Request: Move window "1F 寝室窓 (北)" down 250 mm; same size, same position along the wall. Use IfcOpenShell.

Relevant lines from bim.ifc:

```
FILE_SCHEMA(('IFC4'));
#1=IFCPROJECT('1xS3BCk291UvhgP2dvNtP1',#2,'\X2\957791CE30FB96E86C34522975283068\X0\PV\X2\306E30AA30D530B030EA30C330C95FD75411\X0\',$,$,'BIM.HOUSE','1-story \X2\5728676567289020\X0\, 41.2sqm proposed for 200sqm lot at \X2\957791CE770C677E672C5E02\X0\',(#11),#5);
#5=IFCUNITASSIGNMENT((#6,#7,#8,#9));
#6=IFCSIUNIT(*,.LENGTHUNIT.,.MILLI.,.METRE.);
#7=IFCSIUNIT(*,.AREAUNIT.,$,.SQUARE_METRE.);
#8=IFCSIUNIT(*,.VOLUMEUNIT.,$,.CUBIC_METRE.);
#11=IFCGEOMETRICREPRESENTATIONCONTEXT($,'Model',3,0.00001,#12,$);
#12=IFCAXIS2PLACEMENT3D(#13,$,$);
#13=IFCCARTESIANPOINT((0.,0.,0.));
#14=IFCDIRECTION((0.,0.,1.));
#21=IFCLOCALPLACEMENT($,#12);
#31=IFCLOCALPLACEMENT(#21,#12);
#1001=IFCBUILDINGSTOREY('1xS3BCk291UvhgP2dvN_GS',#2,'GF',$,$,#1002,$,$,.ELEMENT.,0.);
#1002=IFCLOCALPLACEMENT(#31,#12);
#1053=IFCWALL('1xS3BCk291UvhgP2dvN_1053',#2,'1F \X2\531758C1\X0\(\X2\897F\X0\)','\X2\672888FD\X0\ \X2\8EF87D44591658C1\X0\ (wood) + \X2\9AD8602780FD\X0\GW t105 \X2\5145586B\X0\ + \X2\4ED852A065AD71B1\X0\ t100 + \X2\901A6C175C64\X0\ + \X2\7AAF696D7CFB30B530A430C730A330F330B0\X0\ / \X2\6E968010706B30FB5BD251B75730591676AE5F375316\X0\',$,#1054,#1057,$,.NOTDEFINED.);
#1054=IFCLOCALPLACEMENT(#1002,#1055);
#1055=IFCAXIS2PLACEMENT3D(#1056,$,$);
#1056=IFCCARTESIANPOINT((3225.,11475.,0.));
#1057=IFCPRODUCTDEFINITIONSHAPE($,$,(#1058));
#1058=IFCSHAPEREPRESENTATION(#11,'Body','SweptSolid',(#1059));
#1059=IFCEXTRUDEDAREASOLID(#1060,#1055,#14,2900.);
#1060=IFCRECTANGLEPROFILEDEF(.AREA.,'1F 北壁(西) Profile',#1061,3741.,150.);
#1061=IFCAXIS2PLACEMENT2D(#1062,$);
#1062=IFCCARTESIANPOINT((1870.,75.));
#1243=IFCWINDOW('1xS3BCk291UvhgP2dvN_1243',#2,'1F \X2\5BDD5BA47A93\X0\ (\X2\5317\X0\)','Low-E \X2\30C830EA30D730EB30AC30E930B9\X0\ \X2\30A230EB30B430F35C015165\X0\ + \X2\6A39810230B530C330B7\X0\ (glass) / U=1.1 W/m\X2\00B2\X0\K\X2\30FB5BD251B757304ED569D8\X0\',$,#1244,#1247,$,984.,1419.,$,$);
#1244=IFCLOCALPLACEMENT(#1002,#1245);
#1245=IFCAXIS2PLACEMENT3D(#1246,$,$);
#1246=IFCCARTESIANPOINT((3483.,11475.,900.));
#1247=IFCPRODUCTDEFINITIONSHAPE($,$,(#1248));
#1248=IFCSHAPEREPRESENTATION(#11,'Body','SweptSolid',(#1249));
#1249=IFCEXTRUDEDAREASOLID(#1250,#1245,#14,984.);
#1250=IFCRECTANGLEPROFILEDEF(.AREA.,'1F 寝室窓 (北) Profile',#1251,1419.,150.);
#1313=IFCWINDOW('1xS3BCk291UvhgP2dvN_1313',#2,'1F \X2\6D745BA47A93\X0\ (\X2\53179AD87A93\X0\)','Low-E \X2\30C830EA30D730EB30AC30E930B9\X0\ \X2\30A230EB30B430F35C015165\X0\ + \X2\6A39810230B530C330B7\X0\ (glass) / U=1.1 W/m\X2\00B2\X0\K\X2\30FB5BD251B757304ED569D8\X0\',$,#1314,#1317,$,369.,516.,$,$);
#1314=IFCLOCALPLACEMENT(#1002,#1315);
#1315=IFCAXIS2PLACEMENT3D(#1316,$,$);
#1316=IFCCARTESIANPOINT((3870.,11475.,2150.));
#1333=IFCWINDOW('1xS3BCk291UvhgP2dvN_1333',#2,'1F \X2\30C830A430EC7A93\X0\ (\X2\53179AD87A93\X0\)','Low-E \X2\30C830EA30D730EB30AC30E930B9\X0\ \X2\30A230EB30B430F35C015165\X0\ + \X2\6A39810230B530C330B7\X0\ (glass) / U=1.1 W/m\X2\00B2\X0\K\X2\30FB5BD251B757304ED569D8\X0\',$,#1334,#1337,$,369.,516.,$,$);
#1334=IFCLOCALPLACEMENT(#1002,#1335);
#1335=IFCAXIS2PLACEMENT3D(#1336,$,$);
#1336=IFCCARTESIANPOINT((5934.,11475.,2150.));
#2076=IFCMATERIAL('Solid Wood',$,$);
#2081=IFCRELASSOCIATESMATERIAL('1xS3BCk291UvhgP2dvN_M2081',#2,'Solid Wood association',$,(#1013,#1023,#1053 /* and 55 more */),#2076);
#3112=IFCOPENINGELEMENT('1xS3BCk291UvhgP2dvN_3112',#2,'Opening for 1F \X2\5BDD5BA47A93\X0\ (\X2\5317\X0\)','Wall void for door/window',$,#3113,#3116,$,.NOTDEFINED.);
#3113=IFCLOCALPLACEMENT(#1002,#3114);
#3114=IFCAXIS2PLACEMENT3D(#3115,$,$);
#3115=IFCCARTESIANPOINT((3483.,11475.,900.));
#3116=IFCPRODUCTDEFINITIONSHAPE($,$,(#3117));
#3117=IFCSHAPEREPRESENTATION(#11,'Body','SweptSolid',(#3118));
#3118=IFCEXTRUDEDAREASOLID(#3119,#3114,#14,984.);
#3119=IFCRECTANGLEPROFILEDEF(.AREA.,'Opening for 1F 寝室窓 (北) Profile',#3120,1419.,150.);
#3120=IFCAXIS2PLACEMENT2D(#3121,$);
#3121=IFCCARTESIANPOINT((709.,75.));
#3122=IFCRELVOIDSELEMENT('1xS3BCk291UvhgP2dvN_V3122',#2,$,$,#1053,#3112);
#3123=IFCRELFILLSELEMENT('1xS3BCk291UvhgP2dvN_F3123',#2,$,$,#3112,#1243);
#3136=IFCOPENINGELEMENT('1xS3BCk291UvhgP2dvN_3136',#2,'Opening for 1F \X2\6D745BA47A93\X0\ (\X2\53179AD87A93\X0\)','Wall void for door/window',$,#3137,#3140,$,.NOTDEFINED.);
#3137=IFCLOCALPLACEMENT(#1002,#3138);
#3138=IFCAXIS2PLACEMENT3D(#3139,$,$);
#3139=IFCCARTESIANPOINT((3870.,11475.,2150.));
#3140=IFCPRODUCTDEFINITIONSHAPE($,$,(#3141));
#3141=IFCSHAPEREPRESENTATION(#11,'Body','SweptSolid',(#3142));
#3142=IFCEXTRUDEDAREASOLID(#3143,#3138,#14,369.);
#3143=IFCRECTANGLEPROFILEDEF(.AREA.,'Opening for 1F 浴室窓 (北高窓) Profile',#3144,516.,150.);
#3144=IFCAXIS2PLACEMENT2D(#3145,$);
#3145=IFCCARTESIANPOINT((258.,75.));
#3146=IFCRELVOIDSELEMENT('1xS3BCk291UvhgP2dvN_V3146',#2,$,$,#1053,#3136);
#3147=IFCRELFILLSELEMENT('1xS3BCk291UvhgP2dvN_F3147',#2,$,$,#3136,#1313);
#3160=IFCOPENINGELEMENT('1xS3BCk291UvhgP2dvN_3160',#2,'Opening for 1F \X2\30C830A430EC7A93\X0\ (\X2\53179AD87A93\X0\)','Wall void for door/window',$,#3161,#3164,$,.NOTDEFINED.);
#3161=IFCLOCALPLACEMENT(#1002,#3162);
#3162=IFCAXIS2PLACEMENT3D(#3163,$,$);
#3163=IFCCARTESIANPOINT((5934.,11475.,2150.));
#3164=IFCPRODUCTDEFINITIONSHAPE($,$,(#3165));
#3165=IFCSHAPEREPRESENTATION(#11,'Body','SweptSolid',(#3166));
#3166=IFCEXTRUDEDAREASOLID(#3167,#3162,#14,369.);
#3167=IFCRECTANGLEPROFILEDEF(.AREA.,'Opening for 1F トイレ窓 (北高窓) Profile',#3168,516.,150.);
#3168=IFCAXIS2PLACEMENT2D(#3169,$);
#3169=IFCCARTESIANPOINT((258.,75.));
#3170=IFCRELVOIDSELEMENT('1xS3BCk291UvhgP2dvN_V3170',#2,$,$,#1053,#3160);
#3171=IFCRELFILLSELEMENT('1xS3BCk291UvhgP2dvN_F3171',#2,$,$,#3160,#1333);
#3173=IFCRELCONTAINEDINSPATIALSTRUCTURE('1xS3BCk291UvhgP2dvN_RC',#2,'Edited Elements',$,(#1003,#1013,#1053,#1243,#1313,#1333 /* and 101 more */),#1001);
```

```python
import numpy as np
import ifcopenshell
import ifcopenshell.api.geometry
import ifcopenshell.util.placement
import ifcopenshell.util.unit

model = ifcopenshell.open("bim.ifc")
unit_scale = ifcopenshell.util.unit.calculate_unit_scale(model)

window = model.by_guid("1xS3BCk291UvhgP2dvN_1243")
opening = window.FillsVoids[0].RelatingOpeningElement
dz = -0.25 / unit_scale

shift = np.array([0.0, 0.0, dz])
# The window is not placed relative to its opening, so move both.
for product in (opening, window):
    matrix = ifcopenshell.util.placement.get_local_placement(product.ObjectPlacement)
    matrix[:3, 3] += shift
    ifcopenshell.api.geometry.edit_object_placement(model, product=product, matrix=matrix, is_si=False)

print(f"moved by {dz * unit_scale:+.3f} m")

model.write("bim_v2.ifc")
```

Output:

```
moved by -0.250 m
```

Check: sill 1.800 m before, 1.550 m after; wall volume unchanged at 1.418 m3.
